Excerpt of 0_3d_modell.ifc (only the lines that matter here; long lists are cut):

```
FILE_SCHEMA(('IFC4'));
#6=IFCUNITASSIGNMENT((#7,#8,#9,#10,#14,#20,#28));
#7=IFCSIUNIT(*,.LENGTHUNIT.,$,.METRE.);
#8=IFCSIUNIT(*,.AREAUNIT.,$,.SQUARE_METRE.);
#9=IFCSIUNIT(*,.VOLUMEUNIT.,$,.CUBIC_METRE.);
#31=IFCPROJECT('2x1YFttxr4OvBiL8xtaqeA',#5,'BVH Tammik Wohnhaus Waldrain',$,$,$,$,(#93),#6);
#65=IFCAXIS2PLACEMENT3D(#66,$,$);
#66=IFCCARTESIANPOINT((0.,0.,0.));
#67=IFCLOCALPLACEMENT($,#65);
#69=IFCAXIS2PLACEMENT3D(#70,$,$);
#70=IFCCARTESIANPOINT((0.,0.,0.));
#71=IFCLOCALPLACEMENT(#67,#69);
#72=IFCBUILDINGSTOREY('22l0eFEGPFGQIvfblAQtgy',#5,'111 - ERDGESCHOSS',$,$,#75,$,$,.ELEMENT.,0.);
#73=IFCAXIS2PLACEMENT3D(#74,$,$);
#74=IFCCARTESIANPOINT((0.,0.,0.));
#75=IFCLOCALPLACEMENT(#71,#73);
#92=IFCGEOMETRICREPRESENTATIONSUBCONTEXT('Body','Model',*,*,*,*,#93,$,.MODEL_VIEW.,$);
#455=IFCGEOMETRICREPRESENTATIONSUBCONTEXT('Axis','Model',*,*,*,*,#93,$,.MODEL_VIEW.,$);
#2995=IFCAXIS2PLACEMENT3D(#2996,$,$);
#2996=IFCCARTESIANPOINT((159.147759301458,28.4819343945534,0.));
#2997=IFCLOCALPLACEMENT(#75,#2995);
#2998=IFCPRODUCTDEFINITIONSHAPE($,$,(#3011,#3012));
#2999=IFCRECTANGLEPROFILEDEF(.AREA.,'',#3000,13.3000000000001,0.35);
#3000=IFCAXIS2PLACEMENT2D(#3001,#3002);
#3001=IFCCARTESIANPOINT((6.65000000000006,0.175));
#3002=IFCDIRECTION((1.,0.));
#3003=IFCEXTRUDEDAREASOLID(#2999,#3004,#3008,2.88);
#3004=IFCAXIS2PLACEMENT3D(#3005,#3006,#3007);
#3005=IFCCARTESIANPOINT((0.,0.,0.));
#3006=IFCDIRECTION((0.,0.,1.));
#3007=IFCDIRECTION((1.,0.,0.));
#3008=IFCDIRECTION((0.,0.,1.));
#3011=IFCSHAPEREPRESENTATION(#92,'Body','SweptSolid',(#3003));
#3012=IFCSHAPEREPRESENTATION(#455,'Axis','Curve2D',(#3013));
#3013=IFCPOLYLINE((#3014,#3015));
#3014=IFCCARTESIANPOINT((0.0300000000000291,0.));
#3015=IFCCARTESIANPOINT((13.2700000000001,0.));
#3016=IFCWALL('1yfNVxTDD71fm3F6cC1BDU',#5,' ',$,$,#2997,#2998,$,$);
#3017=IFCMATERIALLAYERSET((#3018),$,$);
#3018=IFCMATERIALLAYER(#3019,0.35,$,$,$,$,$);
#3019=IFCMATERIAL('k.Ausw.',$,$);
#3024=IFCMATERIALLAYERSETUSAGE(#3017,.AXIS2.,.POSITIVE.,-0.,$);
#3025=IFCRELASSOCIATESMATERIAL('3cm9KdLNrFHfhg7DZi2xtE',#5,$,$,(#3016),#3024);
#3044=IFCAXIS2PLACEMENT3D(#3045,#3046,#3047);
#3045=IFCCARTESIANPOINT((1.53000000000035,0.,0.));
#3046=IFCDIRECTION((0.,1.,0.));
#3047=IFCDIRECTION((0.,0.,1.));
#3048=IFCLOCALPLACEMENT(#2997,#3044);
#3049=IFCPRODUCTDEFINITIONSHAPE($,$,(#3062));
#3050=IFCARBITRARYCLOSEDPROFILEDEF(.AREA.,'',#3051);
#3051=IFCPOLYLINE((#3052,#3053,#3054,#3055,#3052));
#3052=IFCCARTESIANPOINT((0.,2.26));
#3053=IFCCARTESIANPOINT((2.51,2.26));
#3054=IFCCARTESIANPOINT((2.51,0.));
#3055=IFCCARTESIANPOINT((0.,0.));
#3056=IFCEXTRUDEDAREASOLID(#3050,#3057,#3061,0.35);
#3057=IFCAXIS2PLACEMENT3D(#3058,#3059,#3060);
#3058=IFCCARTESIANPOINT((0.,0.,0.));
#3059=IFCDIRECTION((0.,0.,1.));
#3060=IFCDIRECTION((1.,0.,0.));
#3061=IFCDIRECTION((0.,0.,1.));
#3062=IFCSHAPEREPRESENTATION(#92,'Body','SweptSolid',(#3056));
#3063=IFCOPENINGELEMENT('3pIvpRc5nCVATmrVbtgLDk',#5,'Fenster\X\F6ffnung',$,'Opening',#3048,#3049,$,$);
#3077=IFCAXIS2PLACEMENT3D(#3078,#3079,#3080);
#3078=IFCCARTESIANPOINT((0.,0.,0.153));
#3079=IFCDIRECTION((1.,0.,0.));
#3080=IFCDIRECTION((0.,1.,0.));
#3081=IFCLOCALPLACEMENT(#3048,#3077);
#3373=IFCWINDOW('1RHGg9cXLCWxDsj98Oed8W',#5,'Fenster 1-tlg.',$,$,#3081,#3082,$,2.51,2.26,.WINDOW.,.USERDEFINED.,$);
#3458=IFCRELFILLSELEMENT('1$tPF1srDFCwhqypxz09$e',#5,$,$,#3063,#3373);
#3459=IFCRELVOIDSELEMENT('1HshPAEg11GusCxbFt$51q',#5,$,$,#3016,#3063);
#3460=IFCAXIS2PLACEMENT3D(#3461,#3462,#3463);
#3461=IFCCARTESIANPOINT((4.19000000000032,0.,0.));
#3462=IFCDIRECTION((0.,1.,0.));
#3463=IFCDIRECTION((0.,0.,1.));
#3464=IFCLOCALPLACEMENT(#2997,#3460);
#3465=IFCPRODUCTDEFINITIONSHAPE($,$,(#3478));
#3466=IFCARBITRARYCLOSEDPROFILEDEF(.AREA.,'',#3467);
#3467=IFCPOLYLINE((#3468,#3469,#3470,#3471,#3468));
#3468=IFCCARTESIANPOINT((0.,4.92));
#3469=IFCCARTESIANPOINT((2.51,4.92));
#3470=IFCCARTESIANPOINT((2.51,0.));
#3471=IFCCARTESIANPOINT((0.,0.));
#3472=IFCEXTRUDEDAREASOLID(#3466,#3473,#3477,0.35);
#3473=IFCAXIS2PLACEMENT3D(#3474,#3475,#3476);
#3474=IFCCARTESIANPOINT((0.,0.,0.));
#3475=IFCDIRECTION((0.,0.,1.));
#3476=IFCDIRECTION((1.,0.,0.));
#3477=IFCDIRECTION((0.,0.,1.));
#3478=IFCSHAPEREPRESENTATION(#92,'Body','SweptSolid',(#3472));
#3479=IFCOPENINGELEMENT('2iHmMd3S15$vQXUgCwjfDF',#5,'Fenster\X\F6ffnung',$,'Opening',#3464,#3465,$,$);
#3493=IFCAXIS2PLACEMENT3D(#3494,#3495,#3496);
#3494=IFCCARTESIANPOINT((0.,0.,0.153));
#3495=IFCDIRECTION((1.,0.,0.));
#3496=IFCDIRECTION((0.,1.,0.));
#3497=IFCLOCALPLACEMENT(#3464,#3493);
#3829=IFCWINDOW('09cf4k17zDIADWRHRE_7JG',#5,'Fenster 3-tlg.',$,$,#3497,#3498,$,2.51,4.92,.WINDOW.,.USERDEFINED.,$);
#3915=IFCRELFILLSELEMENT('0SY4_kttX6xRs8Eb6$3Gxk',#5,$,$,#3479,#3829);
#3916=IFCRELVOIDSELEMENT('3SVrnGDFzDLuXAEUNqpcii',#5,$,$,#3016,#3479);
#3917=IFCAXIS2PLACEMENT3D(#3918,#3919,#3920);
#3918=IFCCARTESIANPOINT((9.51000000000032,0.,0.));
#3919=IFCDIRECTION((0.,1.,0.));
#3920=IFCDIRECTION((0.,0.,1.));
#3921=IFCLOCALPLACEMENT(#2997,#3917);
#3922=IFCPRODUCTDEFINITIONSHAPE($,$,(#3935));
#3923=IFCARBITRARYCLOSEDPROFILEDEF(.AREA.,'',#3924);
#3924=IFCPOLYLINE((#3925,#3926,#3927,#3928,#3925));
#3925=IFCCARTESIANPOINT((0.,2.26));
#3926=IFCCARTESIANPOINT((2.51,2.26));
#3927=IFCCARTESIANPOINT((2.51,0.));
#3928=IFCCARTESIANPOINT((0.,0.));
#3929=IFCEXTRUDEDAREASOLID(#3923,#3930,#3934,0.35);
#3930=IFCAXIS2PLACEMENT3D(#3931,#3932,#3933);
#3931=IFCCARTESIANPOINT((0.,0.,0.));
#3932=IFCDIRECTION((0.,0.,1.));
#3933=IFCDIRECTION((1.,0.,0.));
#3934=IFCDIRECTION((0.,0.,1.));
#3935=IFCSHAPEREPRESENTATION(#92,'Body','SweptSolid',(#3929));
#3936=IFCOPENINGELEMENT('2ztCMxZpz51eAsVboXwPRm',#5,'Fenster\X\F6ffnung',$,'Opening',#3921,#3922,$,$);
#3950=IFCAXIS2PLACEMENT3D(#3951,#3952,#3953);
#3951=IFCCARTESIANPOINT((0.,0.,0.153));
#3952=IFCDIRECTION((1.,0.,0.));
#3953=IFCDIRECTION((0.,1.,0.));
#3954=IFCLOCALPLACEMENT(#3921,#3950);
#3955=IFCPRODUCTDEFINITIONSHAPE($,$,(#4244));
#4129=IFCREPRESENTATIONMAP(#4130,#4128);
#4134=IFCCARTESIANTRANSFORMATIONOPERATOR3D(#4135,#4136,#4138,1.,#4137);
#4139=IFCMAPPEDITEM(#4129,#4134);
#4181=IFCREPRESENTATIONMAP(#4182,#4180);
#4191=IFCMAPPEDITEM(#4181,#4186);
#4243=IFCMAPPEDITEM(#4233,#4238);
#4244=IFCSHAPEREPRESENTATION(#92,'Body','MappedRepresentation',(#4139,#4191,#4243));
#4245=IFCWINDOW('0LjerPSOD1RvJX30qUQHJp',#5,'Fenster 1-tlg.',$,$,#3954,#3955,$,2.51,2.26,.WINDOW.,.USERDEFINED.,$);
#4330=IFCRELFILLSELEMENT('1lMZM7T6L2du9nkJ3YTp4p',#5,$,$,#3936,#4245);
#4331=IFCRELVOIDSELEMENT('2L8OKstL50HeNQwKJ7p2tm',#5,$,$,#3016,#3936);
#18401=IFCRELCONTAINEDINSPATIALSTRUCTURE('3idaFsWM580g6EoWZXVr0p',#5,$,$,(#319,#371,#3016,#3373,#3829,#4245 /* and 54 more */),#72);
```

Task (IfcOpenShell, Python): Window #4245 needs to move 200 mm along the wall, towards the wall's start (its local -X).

```python
import ifcopenshell
import ifcopenshell.api.geometry
import ifcopenshell.util.placement
import ifcopenshell.util.unit

model = ifcopenshell.open("0_3d_modell.ifc")
unit_scale = ifcopenshell.util.unit.calculate_unit_scale(model)

window = model.by_id(4245)
opening = window.FillsVoids[0].RelatingOpeningElement
wall = opening.VoidsElements[0].RelatingBuildingElement

wall_matrix = ifcopenshell.util.placement.get_local_placement(wall.ObjectPlacement)
shift = wall_matrix[:3, 0] * -0.2 / unit_scale
before = ifcopenshell.util.placement.get_local_placement(window.ObjectPlacement)[:3, 3].copy()

# The window is placed relative to its opening, so it follows when the opening moves.
matrix = ifcopenshell.util.placement.get_local_placement(opening.ObjectPlacement)
matrix[:3, 3] += shift
ifcopenshell.api.geometry.edit_object_placement(
    model, product=opening, matrix=matrix, is_si=False, should_transform_children=True
)

after = ifcopenshell.util.placement.get_local_placement(window.ObjectPlacement)[:3, 3]
print("window moved by", (after - before).round(3) + 0.0)

model.write("0_3d_modell_updated.ifc")
```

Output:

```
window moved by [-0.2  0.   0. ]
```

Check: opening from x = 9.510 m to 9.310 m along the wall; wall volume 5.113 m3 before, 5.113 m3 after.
